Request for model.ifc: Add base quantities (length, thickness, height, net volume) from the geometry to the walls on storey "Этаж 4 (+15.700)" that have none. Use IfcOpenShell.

First a look at what the model holds.

```python
import ifcopenshell
import ifcopenshell.util.element
import ifcopenshell.util.unit

model = ifcopenshell.open("model.ifc")
print(model.schema)
for unit_type in ("LENGTHUNIT", "AREAUNIT", "VOLUMEUNIT"):
    print(unit_type, ifcopenshell.util.unit.calculate_unit_scale(model, unit_type))
storey = next(s for s in model.by_type("IfcBuildingStorey") if s.Name == "Этаж 4 (+15.700)")
walls = [e for e in ifcopenshell.util.element.get_decomposition(storey) if e.is_a("IfcWall")]
for e in sorted(walls, key=lambda e: e.id()):
    print(e.id(), e.is_a(), e.Name, list(ifcopenshell.util.element.get_psets(e, qtos_only=True)), sep=" | ")
```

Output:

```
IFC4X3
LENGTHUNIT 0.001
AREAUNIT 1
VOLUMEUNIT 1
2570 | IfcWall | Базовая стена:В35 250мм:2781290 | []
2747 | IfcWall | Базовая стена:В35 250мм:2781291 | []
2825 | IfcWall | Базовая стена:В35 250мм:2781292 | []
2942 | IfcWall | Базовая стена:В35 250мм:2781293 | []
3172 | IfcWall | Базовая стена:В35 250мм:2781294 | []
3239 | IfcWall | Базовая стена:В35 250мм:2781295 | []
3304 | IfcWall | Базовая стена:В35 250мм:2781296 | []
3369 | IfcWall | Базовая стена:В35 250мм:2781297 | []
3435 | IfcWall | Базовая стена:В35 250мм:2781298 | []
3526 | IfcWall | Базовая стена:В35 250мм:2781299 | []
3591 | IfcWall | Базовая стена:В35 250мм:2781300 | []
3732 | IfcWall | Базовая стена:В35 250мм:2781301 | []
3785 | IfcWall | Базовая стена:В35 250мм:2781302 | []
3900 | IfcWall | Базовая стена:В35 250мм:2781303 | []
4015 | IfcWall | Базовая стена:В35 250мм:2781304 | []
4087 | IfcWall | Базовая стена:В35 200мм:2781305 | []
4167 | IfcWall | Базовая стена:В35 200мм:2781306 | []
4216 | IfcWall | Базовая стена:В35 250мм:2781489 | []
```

```python
import ifcopenshell
import ifcopenshell.api.pset
import ifcopenshell.geom
import ifcopenshell.util.element
import ifcopenshell.util.shape
import ifcopenshell.util.unit

model = ifcopenshell.open("model.ifc")
unit_scale = ifcopenshell.util.unit.calculate_unit_scale(model)
volume_scale = ifcopenshell.util.unit.calculate_unit_scale(model, "VOLUMEUNIT")
settings = ifcopenshell.geom.settings()

storey = next(s for s in model.by_type("IfcBuildingStorey") if s.Name == "Этаж 4 (+15.700)")
walls = [e for e in ifcopenshell.util.element.get_decomposition(storey) if e.is_a("IfcWall")]

for e in sorted(walls, key=lambda e: e.id()):
    if ifcopenshell.util.element.get_psets(e, qtos_only=True, should_inherit=False):
        continue
    # Geometry comes back in metres, in the element's own axes.
    shape = ifcopenshell.geom.create_shape(settings, e)
    values = {
        "Length": ifcopenshell.util.shape.get_x(shape.geometry) / unit_scale,
        "Width": ifcopenshell.util.shape.get_y(shape.geometry) / unit_scale,
        "Height": ifcopenshell.util.shape.get_z(shape.geometry) / unit_scale,
        "NetVolume": ifcopenshell.util.shape.get_volume(shape.geometry) / volume_scale,
    }
    qto = ifcopenshell.api.pset.add_qto(model, product=e, name="Qto_WallBaseQuantities")
    ifcopenshell.api.pset.edit_qto(model, qto=qto, properties=values)
    print(e.id(), {k: round(v, 3) for k, v in values.items()})

model.write("model_updated.ifc")
```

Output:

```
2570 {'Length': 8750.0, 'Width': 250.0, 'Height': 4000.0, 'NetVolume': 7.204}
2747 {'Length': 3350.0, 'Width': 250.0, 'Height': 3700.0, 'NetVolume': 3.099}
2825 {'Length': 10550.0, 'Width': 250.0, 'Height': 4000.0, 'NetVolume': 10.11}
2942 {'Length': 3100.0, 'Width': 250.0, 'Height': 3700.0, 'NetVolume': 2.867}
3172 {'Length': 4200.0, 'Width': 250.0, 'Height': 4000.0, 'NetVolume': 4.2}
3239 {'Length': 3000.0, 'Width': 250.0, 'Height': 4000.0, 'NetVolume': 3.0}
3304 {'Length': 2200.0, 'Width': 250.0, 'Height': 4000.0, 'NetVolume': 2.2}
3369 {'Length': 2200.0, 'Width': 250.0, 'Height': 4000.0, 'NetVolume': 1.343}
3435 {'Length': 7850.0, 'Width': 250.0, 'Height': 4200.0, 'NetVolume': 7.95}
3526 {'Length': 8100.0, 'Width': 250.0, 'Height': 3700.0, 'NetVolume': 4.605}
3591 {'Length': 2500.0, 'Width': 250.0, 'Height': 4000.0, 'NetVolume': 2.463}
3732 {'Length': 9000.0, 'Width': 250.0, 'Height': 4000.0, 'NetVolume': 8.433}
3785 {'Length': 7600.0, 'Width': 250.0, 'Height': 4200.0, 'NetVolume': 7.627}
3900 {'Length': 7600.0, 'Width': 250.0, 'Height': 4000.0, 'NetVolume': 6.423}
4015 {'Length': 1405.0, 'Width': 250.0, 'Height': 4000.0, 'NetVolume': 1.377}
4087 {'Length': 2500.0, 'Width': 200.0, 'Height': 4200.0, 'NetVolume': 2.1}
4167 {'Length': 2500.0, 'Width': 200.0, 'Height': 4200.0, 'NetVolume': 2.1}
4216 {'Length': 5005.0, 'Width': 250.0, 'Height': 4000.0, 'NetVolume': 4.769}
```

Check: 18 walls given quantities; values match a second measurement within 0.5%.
